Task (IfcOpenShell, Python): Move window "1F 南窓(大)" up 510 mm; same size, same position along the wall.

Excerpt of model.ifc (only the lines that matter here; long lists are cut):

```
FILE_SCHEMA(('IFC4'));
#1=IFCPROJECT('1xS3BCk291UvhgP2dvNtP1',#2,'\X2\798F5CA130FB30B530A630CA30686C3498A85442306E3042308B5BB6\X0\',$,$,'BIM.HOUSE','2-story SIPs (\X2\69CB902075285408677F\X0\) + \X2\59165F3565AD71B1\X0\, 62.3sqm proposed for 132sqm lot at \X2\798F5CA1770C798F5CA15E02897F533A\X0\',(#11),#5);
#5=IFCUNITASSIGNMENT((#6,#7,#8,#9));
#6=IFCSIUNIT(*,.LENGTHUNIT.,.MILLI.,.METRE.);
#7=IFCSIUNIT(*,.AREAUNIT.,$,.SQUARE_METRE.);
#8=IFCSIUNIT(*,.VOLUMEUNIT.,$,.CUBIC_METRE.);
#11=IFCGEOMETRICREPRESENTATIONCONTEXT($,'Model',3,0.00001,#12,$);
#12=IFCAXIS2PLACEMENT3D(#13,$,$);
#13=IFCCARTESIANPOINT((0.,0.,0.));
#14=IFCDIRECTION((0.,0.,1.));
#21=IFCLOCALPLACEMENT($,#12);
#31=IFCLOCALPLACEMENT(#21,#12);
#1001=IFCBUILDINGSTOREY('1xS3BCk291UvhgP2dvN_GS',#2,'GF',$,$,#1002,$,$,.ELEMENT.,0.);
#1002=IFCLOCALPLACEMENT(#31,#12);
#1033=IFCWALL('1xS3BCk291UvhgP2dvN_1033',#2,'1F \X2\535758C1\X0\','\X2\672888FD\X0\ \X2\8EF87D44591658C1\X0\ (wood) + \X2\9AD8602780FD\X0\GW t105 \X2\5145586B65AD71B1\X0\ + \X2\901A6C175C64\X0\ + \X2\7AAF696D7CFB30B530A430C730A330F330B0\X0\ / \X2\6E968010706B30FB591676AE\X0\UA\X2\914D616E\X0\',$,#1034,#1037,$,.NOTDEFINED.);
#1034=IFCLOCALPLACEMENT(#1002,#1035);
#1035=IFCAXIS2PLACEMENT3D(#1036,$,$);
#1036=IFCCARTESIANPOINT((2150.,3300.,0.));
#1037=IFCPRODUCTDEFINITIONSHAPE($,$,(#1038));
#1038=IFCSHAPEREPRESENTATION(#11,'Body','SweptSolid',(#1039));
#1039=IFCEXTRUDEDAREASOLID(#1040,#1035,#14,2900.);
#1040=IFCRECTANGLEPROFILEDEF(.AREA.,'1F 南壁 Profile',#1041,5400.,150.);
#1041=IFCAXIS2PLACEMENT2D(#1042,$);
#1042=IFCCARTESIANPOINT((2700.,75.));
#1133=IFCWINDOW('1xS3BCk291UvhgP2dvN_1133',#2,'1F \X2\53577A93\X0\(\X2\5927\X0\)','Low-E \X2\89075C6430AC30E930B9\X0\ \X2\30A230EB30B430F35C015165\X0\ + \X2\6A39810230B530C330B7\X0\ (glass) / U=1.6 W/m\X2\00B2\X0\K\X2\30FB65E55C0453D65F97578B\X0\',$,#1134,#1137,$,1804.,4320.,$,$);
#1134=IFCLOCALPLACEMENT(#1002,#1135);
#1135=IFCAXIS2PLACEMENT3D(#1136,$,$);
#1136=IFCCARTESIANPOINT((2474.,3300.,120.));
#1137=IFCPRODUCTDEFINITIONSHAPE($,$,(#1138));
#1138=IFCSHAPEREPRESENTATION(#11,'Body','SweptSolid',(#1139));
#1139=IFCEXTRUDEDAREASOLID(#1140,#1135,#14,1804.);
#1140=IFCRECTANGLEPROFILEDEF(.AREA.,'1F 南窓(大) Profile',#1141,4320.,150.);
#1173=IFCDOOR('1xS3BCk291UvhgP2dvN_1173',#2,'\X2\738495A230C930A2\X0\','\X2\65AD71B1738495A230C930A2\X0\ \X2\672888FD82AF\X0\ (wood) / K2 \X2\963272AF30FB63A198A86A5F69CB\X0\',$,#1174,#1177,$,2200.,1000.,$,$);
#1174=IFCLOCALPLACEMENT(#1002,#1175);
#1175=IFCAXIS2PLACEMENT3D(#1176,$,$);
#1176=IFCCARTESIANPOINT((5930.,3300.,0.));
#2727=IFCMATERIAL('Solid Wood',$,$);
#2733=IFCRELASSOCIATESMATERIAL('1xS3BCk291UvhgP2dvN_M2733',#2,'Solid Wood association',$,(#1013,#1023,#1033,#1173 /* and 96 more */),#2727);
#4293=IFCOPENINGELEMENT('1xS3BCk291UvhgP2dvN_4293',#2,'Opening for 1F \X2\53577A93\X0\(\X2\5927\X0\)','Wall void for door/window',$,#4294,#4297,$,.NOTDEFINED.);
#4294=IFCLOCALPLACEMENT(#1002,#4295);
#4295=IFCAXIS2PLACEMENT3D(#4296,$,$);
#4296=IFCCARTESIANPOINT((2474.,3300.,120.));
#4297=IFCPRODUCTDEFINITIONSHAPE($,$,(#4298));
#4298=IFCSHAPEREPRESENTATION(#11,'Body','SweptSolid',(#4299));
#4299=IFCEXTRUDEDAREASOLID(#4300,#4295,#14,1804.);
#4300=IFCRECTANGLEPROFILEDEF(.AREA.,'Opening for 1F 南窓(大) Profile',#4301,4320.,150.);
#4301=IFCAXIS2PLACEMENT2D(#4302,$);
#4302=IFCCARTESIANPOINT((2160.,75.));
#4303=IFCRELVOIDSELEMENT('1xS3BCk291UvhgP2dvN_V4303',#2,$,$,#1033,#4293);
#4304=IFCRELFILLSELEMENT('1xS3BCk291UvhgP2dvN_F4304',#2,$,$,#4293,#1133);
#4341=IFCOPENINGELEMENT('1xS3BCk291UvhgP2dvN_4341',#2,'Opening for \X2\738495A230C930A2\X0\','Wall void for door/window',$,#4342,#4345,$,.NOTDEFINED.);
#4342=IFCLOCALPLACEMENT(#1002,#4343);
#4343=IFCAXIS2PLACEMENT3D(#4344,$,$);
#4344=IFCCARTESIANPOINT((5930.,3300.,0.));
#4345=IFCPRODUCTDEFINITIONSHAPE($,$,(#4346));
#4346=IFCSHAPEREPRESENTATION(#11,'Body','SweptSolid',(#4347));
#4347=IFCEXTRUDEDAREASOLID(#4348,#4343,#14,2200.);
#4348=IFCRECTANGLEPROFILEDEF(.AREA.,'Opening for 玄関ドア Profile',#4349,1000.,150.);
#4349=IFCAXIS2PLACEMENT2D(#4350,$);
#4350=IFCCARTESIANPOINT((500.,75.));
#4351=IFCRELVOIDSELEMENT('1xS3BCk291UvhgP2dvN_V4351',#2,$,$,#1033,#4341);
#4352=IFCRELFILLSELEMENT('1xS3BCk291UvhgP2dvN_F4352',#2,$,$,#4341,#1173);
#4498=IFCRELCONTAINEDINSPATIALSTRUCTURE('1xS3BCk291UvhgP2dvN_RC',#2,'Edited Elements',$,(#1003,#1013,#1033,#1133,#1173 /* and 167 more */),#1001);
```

```python
import numpy as np
import ifcopenshell
import ifcopenshell.api.geometry
import ifcopenshell.util.placement
import ifcopenshell.util.unit

model = ifcopenshell.open("model.ifc")
unit_scale = ifcopenshell.util.unit.calculate_unit_scale(model)

window = model.by_id(1133)
opening = window.FillsVoids[0].RelatingOpeningElement
dz = 0.51 / unit_scale

shift = np.array([0.0, 0.0, dz])
# The window is not placed relative to its opening, so move both.
for product in (opening, window):
    matrix = ifcopenshell.util.placement.get_local_placement(product.ObjectPlacement)
    matrix[:3, 3] += shift
    ifcopenshell.api.geometry.edit_object_placement(model, product=product, matrix=matrix, is_si=False)

print(f"moved by {dz * unit_scale:+.3f} m")

model.write("model_v2.ifc")
```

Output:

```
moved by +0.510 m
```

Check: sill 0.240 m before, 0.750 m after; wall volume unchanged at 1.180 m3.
